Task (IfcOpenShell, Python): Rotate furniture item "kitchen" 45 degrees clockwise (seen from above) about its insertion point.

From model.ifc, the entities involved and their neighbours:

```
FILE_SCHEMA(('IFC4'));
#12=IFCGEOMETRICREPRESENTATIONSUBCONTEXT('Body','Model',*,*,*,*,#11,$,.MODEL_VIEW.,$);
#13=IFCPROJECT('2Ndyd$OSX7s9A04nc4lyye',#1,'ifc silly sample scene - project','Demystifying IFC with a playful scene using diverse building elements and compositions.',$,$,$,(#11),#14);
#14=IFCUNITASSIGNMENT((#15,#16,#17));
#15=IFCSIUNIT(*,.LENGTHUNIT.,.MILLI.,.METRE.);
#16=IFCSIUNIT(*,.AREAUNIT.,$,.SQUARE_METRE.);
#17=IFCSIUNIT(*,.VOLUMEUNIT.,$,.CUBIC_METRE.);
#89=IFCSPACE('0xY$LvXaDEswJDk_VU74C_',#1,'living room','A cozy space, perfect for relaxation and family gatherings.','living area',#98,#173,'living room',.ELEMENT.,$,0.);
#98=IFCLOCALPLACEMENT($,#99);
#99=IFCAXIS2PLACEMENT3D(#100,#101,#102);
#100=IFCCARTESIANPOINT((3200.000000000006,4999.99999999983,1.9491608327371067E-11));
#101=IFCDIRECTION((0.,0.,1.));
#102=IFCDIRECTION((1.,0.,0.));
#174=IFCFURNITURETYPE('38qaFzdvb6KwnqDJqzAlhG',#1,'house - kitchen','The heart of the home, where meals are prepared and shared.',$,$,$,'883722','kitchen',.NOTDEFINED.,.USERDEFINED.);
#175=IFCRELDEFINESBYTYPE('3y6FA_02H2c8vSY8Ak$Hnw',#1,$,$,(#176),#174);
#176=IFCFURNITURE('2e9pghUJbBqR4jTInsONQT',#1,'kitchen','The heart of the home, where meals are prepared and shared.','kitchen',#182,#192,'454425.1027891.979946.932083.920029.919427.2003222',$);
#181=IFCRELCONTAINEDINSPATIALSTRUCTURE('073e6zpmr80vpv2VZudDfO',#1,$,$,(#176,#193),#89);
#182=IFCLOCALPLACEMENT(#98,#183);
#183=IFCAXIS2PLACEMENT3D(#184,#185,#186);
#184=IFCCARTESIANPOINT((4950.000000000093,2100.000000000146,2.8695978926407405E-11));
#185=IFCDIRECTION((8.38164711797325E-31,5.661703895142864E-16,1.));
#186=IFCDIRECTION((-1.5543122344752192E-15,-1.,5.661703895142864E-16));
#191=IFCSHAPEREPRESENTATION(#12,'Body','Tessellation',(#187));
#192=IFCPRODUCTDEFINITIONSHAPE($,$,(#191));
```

```python
import ifcopenshell
import ifcopenshell.api.geometry
import ifcopenshell.util.placement

model = ifcopenshell.open("model.ifc")

item = model.by_guid("2e9pghUJbBqR4jTInsONQT")
matrix = ifcopenshell.util.placement.get_local_placement(item.ObjectPlacement)
matrix = matrix @ ifcopenshell.util.placement.rotation(-45, "Z")
ifcopenshell.api.geometry.edit_object_placement(model, product=item, matrix=matrix, is_si=False)

print(ifcopenshell.util.placement.get_local_placement(item.ObjectPlacement).round(3) + 0.0)

model.write("model_rev.ifc")
```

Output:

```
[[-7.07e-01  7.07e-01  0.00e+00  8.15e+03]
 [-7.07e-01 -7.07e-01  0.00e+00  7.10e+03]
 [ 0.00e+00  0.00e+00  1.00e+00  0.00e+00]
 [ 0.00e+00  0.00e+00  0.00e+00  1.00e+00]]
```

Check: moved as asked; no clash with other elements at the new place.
